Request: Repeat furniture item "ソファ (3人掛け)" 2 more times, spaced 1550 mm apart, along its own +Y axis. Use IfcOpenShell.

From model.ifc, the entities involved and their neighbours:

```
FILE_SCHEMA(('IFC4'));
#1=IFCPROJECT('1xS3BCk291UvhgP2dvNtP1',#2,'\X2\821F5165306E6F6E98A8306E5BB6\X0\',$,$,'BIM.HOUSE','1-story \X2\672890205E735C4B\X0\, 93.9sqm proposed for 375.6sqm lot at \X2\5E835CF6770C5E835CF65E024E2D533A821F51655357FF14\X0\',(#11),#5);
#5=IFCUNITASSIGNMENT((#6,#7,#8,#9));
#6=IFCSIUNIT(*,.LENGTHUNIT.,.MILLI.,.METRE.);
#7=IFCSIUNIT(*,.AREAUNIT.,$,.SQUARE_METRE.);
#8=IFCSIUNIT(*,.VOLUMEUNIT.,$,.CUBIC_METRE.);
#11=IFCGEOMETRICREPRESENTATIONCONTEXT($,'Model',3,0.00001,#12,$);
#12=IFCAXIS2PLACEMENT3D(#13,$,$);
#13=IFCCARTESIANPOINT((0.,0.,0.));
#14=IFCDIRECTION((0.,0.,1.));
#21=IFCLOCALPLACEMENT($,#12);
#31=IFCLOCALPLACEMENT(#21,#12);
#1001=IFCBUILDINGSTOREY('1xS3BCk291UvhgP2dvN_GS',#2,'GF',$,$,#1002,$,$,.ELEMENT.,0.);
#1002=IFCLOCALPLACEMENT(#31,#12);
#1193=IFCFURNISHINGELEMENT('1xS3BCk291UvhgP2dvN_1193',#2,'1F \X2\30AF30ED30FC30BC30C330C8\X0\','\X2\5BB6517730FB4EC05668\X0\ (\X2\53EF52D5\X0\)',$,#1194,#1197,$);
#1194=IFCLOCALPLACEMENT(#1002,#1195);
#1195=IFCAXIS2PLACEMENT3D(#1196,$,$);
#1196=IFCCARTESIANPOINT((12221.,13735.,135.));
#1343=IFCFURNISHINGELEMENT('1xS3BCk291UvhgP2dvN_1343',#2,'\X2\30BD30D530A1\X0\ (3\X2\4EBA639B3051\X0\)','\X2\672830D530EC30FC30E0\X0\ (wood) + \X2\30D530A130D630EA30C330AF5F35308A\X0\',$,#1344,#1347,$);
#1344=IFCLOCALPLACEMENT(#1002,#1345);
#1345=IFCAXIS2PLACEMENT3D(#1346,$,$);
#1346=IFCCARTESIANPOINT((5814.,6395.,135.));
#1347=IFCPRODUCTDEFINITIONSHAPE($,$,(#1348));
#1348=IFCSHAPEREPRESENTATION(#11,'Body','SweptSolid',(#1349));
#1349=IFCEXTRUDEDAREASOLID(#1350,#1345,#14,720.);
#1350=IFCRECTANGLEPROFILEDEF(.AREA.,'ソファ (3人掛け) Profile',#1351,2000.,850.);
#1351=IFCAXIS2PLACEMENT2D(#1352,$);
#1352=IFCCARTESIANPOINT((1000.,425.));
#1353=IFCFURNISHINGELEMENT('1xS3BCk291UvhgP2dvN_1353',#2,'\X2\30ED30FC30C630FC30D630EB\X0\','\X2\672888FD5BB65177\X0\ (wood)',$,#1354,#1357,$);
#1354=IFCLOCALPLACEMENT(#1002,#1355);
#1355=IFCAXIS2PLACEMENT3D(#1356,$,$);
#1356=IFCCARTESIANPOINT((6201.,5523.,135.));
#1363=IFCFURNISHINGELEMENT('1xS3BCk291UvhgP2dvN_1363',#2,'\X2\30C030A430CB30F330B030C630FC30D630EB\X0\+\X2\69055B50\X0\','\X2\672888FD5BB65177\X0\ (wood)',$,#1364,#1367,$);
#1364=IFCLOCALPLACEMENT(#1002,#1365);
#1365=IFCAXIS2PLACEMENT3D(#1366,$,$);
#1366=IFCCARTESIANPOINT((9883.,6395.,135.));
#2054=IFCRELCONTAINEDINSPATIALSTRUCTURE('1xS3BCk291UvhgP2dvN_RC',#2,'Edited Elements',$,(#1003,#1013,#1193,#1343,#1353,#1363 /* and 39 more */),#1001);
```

```python
import ifcopenshell
import ifcopenshell.api.geometry
import ifcopenshell.api.root
import ifcopenshell.util.element
import ifcopenshell.util.placement
import ifcopenshell.util.unit

model = ifcopenshell.open("model.ifc")
unit_scale = ifcopenshell.util.unit.calculate_unit_scale(model)


def reuse_history(source, copy):
    """copy_class also copies each property set's owner history, people and application; keep the originals."""
    for rel in copy.IsDefinedBy:
        if rel.is_a("IfcRelDefinesByProperties") and (history := rel.RelatingPropertyDefinition.OwnerHistory):
            rel.RelatingPropertyDefinition.OwnerHistory = source.OwnerHistory
            ifcopenshell.util.element.remove_deep2(model, history)


source = model.by_guid("1xS3BCk291UvhgP2dvN_1343")
base = ifcopenshell.util.placement.get_local_placement(source.ObjectPlacement)
step = base[:3, 1] * 1.55 / unit_scale

for i in range(1, 3):
    copy = ifcopenshell.api.root.copy_class(model, product=source)
    copy.Representation = ifcopenshell.util.element.copy_deep(
        model, source.Representation, exclude=["IfcGeometricRepresentationContext", "IfcRepresentationMap"]
    )
    reuse_history(source, copy)
    matrix = base.copy()
    matrix[:3, 3] += i * step
    print("added at", matrix[:3, 3].round(3) + 0.0)
    ifcopenshell.api.geometry.edit_object_placement(model, product=copy, matrix=matrix, is_si=False)

model.write("model_edited.ifc")
```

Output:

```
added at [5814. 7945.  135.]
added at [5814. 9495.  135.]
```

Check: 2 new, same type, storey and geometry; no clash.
